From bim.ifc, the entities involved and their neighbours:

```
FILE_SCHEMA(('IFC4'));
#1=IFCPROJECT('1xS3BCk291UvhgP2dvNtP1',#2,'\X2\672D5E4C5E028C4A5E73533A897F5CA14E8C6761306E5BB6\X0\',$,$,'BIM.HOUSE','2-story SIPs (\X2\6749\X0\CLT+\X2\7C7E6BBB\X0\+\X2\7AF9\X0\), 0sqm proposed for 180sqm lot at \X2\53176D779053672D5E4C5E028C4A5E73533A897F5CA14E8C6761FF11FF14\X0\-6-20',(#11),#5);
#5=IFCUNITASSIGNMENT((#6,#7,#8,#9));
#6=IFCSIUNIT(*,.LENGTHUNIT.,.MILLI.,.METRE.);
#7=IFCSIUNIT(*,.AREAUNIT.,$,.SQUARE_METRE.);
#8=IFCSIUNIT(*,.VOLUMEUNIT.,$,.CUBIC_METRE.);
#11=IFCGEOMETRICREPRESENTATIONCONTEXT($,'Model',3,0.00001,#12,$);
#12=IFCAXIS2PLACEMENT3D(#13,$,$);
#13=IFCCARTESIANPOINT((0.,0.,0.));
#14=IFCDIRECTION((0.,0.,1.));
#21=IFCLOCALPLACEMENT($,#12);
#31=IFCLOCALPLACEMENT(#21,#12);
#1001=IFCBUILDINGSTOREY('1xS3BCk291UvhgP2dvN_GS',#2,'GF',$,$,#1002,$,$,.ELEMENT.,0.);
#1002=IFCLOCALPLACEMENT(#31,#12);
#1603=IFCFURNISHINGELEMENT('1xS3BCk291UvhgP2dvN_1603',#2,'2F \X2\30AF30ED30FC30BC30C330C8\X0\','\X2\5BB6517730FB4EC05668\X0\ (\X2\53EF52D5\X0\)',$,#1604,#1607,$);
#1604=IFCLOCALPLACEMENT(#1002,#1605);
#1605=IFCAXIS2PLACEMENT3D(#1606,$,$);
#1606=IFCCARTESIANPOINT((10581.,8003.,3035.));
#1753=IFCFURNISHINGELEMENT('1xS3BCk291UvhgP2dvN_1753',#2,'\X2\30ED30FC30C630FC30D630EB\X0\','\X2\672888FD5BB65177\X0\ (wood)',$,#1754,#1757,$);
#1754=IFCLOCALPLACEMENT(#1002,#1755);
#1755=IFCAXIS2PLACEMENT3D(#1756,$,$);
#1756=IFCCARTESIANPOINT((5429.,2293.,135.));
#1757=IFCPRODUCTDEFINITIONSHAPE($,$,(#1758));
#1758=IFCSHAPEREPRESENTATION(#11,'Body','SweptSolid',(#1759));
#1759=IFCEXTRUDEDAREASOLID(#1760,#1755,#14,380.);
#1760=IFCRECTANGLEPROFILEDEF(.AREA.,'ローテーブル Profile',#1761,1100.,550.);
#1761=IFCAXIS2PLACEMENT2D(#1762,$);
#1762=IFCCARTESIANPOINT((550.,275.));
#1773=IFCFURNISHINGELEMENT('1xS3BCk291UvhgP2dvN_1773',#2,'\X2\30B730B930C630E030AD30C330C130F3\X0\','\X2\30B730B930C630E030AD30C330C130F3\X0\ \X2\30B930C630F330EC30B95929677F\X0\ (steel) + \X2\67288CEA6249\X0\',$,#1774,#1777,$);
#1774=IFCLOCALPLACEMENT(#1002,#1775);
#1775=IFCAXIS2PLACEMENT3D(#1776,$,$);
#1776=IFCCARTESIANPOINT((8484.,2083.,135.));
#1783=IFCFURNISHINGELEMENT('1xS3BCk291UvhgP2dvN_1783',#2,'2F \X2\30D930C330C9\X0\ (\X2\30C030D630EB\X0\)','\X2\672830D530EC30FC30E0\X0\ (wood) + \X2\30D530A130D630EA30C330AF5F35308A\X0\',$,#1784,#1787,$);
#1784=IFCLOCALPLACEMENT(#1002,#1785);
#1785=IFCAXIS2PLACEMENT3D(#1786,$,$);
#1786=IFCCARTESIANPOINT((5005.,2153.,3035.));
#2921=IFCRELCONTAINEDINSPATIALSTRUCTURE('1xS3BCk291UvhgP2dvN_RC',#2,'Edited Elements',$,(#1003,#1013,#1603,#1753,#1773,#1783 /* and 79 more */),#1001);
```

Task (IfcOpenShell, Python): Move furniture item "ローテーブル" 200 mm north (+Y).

```python
import ifcopenshell
import ifcopenshell.api.geometry
import ifcopenshell.util.placement

model = ifcopenshell.open("bim.ifc")

item = model.by_id(1753)
matrix = ifcopenshell.util.placement.get_local_placement(item.ObjectPlacement)
matrix[1, 3] += 200.0
ifcopenshell.api.geometry.edit_object_placement(model, product=item, matrix=matrix, is_si=False)

print(ifcopenshell.util.placement.get_local_placement(item.ObjectPlacement).round(3) + 0.0)

model.write("bim_v2.ifc")
```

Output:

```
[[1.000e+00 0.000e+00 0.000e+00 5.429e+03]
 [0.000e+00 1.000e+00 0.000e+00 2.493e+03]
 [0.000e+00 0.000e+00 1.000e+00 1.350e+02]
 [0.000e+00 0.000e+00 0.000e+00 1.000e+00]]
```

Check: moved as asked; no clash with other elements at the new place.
